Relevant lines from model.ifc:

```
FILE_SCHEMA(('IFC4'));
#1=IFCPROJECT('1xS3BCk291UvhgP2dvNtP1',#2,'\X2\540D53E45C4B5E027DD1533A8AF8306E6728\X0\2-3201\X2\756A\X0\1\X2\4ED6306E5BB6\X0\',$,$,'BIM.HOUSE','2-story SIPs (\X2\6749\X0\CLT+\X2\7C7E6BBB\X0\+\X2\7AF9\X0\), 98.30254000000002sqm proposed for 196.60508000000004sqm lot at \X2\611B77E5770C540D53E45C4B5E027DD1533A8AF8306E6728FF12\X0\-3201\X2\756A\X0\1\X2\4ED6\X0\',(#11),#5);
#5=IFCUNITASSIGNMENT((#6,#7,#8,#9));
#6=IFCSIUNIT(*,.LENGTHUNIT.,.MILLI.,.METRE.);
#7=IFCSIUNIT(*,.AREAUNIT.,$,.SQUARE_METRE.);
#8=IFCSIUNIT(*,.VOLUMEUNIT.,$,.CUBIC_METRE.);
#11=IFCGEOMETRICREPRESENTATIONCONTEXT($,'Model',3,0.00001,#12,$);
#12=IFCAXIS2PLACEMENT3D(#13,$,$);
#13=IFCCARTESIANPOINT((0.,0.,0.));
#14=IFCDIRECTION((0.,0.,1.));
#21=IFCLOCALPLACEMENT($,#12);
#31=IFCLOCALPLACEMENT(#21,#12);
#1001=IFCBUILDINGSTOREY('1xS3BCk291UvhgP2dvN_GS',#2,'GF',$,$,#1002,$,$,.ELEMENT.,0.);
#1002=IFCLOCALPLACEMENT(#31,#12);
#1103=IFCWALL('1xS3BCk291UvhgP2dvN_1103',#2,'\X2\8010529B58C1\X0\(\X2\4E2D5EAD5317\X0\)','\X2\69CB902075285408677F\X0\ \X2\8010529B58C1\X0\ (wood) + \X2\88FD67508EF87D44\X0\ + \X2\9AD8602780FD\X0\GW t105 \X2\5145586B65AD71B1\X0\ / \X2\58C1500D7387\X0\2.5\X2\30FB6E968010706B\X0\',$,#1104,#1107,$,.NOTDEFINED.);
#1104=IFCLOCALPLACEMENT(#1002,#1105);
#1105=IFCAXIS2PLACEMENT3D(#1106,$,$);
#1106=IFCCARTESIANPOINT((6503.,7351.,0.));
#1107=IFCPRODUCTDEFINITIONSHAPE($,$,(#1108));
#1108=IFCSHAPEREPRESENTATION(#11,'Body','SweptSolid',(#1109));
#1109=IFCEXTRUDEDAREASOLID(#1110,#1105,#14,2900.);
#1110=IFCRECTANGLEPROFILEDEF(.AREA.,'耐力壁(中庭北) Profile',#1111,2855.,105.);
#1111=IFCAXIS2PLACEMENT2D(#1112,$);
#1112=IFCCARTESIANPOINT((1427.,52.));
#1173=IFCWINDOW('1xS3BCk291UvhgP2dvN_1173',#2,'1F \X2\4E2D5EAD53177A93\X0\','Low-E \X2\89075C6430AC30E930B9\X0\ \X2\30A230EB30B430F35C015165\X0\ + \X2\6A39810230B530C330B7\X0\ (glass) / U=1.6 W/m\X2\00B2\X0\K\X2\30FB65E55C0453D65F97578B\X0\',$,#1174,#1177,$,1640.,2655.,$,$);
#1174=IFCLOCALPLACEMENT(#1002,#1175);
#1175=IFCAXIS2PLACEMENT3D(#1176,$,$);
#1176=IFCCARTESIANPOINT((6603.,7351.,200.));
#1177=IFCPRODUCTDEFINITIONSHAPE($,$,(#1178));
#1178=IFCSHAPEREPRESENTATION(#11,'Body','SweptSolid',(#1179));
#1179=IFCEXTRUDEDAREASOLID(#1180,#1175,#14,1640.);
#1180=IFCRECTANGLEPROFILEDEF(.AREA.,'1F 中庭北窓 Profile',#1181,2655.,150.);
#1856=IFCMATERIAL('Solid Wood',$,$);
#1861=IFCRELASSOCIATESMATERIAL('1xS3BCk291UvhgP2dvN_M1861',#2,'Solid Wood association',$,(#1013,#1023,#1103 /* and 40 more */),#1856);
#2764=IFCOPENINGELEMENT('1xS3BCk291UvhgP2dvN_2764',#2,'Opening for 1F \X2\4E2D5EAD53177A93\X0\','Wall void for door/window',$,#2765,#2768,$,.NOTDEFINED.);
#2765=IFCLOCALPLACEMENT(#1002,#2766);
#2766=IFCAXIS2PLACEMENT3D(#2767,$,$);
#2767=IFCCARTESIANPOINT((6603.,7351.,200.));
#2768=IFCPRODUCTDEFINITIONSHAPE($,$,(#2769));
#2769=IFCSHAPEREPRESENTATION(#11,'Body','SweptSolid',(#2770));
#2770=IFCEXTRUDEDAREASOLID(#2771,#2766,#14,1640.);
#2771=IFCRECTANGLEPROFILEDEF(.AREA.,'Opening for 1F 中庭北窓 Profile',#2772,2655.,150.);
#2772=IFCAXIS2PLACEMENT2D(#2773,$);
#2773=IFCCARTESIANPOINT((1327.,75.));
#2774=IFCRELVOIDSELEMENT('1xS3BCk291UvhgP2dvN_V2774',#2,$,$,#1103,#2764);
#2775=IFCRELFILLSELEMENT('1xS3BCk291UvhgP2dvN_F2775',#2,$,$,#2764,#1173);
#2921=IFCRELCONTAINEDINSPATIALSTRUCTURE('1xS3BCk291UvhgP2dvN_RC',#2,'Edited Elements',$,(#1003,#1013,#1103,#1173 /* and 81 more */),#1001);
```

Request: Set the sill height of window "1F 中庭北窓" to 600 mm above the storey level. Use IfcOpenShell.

```python
import numpy as np
import ifcopenshell
import ifcopenshell.api.geometry
import ifcopenshell.geom
import ifcopenshell.util.element
import ifcopenshell.util.placement
import ifcopenshell.util.shape
import ifcopenshell.util.unit

model = ifcopenshell.open("model.ifc")
unit_scale = ifcopenshell.util.unit.calculate_unit_scale(model)

window = model.by_id(1173)
opening = window.FillsVoids[0].RelatingOpeningElement
storey = ifcopenshell.util.element.get_container(window, ifc_class="IfcBuildingStorey")
level = ifcopenshell.util.placement.get_local_placement(storey.ObjectPlacement)[2, 3]

# The opening's origin need not be at the sill, so measure its lowest point.
shape = ifcopenshell.geom.create_shape(ifcopenshell.geom.settings(), opening)
bottom = ifcopenshell.util.shape.get_shape_bottom_elevation(shape, shape.geometry) / unit_scale
dz = level + 0.6 / unit_scale - bottom

shift = np.array([0.0, 0.0, dz])
# The window is not placed relative to its opening, so move both.
for product in (opening, window):
    matrix = ifcopenshell.util.placement.get_local_placement(product.ObjectPlacement)
    matrix[:3, 3] += shift
    ifcopenshell.api.geometry.edit_object_placement(model, product=product, matrix=matrix, is_si=False)

print(f"moved by {dz * unit_scale:+.3f} m")

model.write("model_v2.ifc")
```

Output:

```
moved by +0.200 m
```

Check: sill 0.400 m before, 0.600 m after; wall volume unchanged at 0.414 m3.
